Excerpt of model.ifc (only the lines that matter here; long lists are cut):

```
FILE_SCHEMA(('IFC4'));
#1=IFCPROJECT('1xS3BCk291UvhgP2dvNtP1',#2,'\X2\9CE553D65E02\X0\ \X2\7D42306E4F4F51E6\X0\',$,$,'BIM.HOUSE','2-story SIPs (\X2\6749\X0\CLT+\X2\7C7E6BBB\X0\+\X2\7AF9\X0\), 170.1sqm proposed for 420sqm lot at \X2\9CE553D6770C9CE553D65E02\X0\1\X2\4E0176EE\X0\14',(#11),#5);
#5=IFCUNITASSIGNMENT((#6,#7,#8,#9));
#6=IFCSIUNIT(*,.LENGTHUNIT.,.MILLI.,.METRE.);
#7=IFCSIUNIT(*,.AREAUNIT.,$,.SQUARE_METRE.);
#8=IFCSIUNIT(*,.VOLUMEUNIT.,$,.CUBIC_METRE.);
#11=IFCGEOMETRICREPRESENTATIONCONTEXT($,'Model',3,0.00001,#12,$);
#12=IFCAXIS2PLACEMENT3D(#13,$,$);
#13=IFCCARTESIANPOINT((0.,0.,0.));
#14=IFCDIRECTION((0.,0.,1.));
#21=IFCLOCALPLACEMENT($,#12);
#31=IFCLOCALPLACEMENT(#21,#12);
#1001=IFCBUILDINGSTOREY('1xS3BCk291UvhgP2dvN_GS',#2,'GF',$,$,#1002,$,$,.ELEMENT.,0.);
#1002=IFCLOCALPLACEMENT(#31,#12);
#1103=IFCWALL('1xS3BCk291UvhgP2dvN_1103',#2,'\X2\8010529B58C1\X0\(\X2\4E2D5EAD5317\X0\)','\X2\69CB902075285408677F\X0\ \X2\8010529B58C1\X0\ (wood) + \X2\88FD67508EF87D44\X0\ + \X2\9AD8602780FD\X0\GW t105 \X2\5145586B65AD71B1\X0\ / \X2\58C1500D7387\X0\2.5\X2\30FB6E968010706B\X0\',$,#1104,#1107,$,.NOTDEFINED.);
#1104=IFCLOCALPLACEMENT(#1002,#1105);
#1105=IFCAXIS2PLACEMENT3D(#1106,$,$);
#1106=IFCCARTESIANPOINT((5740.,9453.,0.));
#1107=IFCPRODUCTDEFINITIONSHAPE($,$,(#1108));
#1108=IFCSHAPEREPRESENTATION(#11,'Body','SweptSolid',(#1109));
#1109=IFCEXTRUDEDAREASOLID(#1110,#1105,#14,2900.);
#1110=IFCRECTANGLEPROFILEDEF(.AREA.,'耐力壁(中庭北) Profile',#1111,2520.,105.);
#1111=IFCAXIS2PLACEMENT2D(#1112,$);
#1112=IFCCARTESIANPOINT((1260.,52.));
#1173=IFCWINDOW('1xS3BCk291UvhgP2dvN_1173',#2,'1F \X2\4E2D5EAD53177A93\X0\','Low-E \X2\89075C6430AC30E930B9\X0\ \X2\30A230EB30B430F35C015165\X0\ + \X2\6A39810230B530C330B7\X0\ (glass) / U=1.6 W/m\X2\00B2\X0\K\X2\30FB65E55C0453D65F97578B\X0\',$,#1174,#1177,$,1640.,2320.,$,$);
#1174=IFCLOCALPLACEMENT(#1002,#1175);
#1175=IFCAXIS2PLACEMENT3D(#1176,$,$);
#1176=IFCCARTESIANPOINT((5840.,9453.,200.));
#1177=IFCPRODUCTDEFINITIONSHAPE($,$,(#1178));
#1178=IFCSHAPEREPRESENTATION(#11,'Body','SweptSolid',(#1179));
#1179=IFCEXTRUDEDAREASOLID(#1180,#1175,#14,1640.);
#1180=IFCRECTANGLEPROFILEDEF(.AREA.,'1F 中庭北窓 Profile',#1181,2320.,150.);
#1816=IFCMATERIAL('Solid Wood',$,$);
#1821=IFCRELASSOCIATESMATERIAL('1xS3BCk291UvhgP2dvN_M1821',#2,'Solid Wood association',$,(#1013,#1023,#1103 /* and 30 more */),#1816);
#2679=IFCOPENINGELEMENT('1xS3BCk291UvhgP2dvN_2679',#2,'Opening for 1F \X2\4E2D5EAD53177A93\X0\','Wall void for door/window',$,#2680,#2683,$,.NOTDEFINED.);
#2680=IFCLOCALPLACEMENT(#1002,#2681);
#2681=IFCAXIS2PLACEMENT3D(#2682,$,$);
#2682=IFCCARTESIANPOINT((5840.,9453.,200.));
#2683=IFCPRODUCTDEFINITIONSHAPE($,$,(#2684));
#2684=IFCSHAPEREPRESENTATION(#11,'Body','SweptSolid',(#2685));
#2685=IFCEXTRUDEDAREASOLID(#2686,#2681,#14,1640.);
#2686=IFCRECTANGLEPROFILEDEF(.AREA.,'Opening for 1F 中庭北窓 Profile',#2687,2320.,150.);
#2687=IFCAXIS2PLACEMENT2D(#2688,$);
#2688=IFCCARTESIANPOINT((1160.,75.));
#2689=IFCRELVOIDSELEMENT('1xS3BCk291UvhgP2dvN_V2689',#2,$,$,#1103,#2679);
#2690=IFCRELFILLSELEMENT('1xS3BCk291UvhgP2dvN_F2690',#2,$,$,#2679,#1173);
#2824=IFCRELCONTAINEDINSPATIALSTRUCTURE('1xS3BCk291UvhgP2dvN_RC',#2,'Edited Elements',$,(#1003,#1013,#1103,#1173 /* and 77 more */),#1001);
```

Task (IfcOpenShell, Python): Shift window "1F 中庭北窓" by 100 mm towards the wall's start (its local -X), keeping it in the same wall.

```python
import ifcopenshell
import ifcopenshell.api.geometry
import ifcopenshell.util.placement

model = ifcopenshell.open("model.ifc")

window = model.by_guid("1xS3BCk291UvhgP2dvN_1173")
opening = window.FillsVoids[0].RelatingOpeningElement
wall = opening.VoidsElements[0].RelatingBuildingElement

wall_matrix = ifcopenshell.util.placement.get_local_placement(wall.ObjectPlacement)
shift = wall_matrix[:3, 0] * -100.0
before = ifcopenshell.util.placement.get_local_placement(window.ObjectPlacement)[:3, 3].copy()

# The window is not placed relative to its opening, so move both.
for product in (opening, window):
    matrix = ifcopenshell.util.placement.get_local_placement(product.ObjectPlacement)
    matrix[:3, 3] += shift
    ifcopenshell.api.geometry.edit_object_placement(model, product=product, matrix=matrix, is_si=False)

after = ifcopenshell.util.placement.get_local_placement(window.ObjectPlacement)[:3, 3]
print("window moved by", (after - before).round(3) + 0.0)

model.write("model_edited.ifc")
```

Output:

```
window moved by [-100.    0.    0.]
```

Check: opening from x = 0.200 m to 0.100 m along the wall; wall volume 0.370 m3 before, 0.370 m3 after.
